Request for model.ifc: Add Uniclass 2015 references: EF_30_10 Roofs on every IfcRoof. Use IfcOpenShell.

First a look at what the model holds.

```python
import ifcopenshell

model = ifcopenshell.open("model.ifc")
print(model.schema)
print("classifications:", [c.Name for c in model.by_type("IfcClassification")])
for ifc_class in ("IfcDoor", "IfcRoof", "IfcStair", "IfcWall", "IfcWindow"):
    print(ifc_class, len(model.by_type(ifc_class)))
```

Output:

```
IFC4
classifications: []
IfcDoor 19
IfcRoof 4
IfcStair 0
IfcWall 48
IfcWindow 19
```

```python
import ifcopenshell
import ifcopenshell.api.classification

model = ifcopenshell.open("model.ifc")

system = ifcopenshell.api.classification.add_classification(model, classification="Uniclass 2015")

codes = {
    "IfcRoof": ("EF_30_10", "Roofs"),
}
for ifc_class, (code, name) in codes.items():
    products = model.by_type(ifc_class)
    ifcopenshell.api.classification.add_reference(
        model, products=products, classification=system, identification=code, name=name
    )
    print(code, len(products))

model.write("model-out.ifc")
```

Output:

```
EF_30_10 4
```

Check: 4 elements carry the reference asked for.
